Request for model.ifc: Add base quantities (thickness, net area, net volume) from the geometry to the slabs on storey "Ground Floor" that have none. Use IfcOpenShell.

First a look at what the model holds.

```python
import ifcopenshell
import ifcopenshell.util.element
import ifcopenshell.util.unit

model = ifcopenshell.open("model.ifc")
print(model.schema)
for unit_type in ("LENGTHUNIT", "AREAUNIT", "VOLUMEUNIT"):
    print(unit_type, ifcopenshell.util.unit.calculate_unit_scale(model, unit_type))
storey = next(s for s in model.by_type("IfcBuildingStorey") if s.Name == "Ground Floor")
slabs = [e for e in ifcopenshell.util.element.get_decomposition(storey) if e.is_a("IfcSlab")]
for e in sorted(slabs, key=lambda e: e.id()):
    print(e.id(), e.is_a(), e.Name, list(ifcopenshell.util.element.get_psets(e, qtos_only=True)), sep=" | ")
```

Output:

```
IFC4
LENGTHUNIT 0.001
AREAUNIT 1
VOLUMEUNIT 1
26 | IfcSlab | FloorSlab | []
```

```python
import ifcopenshell
import ifcopenshell.api.pset
import ifcopenshell.geom
import ifcopenshell.util.element
import ifcopenshell.util.shape
import ifcopenshell.util.unit

model = ifcopenshell.open("model.ifc")
unit_scale = ifcopenshell.util.unit.calculate_unit_scale(model)
area_scale = ifcopenshell.util.unit.calculate_unit_scale(model, "AREAUNIT")
volume_scale = ifcopenshell.util.unit.calculate_unit_scale(model, "VOLUMEUNIT")
settings = ifcopenshell.geom.settings()

storey = next(s for s in model.by_type("IfcBuildingStorey") if s.Name == "Ground Floor")
slabs = [e for e in ifcopenshell.util.element.get_decomposition(storey) if e.is_a("IfcSlab")]

for e in sorted(slabs, key=lambda e: e.id()):
    if ifcopenshell.util.element.get_psets(e, qtos_only=True, should_inherit=False):
        continue
    # Geometry comes back in metres, in the element's own axes.
    shape = ifcopenshell.geom.create_shape(settings, e)
    values = {
        "Width": ifcopenshell.util.shape.get_z(shape.geometry) / unit_scale,
        "NetArea": ifcopenshell.util.shape.get_footprint_area(shape.geometry) / area_scale,
        "NetVolume": ifcopenshell.util.shape.get_volume(shape.geometry) / volume_scale,
    }
    qto = ifcopenshell.api.pset.add_qto(model, product=e, name="Qto_SlabBaseQuantities")
    ifcopenshell.api.pset.edit_qto(model, qto=qto, properties=values)
    print(e.id(), {k: round(v, 3) for k, v in values.items()})

model.write("model_v2.ifc")
```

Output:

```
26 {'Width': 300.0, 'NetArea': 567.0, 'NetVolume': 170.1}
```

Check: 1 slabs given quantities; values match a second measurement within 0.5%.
